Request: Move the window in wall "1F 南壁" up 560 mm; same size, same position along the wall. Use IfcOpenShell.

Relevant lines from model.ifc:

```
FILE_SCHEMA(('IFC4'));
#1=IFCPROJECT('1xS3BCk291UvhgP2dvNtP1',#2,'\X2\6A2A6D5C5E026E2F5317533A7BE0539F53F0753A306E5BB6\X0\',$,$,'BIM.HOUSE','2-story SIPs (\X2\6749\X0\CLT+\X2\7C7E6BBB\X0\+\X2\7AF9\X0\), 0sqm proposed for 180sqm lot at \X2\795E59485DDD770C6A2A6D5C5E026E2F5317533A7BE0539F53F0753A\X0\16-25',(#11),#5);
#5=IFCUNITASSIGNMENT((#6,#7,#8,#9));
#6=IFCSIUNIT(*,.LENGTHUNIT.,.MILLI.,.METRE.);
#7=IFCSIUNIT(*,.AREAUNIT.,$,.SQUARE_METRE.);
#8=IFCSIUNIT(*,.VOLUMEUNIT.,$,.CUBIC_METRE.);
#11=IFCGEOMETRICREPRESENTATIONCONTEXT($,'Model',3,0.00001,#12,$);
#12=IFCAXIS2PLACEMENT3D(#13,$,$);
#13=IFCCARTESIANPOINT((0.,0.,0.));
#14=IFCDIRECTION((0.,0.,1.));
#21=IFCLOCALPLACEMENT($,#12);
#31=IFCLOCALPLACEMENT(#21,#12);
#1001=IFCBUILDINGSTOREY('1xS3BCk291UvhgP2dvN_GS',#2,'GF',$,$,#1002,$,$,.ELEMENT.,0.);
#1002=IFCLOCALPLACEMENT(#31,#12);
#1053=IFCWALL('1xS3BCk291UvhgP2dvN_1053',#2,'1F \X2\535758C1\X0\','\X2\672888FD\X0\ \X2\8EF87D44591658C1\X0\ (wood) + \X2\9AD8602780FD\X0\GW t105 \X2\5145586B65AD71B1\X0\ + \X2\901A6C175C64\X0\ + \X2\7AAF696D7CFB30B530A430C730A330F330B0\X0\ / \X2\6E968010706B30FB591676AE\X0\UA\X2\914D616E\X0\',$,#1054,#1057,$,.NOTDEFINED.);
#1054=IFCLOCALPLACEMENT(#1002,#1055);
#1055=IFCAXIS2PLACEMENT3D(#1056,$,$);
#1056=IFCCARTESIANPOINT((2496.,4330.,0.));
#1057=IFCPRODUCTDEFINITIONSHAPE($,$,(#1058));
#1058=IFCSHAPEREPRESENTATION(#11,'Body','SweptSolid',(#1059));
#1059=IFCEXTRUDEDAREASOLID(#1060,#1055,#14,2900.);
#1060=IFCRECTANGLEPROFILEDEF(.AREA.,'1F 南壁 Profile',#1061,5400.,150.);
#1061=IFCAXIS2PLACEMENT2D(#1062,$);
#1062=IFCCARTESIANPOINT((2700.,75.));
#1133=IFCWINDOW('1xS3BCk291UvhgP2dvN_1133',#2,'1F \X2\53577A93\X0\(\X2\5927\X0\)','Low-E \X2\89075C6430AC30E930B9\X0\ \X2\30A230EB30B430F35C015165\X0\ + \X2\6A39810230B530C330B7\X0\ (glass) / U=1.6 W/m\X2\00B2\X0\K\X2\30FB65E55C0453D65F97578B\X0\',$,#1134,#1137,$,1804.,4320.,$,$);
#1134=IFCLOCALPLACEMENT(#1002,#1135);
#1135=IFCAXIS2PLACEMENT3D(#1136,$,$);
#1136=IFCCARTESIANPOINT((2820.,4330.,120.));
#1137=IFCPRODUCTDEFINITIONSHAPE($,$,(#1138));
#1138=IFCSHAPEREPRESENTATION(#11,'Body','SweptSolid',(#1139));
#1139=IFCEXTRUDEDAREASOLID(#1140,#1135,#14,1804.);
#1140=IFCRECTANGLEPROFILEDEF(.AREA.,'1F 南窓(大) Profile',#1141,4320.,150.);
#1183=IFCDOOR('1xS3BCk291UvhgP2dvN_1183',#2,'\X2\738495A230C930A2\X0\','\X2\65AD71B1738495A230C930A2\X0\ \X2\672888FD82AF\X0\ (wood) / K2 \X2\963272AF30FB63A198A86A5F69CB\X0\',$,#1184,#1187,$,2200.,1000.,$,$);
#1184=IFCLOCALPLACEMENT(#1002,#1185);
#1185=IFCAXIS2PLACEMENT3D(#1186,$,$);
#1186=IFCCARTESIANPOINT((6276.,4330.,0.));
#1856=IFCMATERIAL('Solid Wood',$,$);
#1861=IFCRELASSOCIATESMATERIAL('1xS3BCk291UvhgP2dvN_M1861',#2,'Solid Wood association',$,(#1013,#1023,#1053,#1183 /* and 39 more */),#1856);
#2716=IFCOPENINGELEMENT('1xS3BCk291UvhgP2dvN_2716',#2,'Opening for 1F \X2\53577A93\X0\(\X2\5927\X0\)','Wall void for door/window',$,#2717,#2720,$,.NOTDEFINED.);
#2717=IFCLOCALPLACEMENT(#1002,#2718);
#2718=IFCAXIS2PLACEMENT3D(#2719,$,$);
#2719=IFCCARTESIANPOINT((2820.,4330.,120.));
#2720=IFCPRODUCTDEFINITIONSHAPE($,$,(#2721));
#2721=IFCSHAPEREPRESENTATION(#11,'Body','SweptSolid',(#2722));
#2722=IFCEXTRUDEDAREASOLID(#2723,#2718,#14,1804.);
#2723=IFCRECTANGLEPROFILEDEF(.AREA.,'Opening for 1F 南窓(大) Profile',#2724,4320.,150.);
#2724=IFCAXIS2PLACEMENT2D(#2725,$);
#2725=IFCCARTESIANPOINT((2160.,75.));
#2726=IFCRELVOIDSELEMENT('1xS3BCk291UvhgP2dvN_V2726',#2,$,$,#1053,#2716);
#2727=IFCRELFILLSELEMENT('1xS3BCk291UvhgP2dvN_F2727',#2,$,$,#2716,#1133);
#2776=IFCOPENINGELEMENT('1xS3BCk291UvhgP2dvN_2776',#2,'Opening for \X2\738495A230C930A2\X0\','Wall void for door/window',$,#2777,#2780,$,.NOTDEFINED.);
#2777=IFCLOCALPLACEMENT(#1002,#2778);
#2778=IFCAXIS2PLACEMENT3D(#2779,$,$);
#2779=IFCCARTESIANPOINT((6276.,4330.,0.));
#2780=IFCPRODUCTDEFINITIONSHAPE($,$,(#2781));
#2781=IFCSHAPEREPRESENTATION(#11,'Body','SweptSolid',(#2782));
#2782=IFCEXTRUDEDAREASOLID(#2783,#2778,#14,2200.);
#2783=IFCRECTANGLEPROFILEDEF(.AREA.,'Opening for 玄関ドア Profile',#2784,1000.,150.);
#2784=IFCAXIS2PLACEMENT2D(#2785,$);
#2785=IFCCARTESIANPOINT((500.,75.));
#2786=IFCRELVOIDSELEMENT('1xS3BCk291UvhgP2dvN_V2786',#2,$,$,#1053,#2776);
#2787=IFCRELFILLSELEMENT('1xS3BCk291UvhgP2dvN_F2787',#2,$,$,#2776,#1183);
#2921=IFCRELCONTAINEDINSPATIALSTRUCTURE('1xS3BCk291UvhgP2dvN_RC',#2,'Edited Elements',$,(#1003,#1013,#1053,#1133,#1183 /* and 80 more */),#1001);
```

```python
import numpy as np
import ifcopenshell
import ifcopenshell.api.geometry
import ifcopenshell.util.placement
import ifcopenshell.util.unit

model = ifcopenshell.open("model.ifc")
unit_scale = ifcopenshell.util.unit.calculate_unit_scale(model)

window = model.by_guid("1xS3BCk291UvhgP2dvN_1133")
opening = window.FillsVoids[0].RelatingOpeningElement
dz = 560.0

shift = np.array([0.0, 0.0, dz])
# The window is not placed relative to its opening, so move both.
for product in (opening, window):
    matrix = ifcopenshell.util.placement.get_local_placement(product.ObjectPlacement)
    matrix[:3, 3] += shift
    ifcopenshell.api.geometry.edit_object_placement(model, product=product, matrix=matrix, is_si=False)

print(f"moved by {dz * unit_scale:+.3f} m")

model.write("model_edited.ifc")
```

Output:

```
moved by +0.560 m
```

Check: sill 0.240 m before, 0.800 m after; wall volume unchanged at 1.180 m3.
